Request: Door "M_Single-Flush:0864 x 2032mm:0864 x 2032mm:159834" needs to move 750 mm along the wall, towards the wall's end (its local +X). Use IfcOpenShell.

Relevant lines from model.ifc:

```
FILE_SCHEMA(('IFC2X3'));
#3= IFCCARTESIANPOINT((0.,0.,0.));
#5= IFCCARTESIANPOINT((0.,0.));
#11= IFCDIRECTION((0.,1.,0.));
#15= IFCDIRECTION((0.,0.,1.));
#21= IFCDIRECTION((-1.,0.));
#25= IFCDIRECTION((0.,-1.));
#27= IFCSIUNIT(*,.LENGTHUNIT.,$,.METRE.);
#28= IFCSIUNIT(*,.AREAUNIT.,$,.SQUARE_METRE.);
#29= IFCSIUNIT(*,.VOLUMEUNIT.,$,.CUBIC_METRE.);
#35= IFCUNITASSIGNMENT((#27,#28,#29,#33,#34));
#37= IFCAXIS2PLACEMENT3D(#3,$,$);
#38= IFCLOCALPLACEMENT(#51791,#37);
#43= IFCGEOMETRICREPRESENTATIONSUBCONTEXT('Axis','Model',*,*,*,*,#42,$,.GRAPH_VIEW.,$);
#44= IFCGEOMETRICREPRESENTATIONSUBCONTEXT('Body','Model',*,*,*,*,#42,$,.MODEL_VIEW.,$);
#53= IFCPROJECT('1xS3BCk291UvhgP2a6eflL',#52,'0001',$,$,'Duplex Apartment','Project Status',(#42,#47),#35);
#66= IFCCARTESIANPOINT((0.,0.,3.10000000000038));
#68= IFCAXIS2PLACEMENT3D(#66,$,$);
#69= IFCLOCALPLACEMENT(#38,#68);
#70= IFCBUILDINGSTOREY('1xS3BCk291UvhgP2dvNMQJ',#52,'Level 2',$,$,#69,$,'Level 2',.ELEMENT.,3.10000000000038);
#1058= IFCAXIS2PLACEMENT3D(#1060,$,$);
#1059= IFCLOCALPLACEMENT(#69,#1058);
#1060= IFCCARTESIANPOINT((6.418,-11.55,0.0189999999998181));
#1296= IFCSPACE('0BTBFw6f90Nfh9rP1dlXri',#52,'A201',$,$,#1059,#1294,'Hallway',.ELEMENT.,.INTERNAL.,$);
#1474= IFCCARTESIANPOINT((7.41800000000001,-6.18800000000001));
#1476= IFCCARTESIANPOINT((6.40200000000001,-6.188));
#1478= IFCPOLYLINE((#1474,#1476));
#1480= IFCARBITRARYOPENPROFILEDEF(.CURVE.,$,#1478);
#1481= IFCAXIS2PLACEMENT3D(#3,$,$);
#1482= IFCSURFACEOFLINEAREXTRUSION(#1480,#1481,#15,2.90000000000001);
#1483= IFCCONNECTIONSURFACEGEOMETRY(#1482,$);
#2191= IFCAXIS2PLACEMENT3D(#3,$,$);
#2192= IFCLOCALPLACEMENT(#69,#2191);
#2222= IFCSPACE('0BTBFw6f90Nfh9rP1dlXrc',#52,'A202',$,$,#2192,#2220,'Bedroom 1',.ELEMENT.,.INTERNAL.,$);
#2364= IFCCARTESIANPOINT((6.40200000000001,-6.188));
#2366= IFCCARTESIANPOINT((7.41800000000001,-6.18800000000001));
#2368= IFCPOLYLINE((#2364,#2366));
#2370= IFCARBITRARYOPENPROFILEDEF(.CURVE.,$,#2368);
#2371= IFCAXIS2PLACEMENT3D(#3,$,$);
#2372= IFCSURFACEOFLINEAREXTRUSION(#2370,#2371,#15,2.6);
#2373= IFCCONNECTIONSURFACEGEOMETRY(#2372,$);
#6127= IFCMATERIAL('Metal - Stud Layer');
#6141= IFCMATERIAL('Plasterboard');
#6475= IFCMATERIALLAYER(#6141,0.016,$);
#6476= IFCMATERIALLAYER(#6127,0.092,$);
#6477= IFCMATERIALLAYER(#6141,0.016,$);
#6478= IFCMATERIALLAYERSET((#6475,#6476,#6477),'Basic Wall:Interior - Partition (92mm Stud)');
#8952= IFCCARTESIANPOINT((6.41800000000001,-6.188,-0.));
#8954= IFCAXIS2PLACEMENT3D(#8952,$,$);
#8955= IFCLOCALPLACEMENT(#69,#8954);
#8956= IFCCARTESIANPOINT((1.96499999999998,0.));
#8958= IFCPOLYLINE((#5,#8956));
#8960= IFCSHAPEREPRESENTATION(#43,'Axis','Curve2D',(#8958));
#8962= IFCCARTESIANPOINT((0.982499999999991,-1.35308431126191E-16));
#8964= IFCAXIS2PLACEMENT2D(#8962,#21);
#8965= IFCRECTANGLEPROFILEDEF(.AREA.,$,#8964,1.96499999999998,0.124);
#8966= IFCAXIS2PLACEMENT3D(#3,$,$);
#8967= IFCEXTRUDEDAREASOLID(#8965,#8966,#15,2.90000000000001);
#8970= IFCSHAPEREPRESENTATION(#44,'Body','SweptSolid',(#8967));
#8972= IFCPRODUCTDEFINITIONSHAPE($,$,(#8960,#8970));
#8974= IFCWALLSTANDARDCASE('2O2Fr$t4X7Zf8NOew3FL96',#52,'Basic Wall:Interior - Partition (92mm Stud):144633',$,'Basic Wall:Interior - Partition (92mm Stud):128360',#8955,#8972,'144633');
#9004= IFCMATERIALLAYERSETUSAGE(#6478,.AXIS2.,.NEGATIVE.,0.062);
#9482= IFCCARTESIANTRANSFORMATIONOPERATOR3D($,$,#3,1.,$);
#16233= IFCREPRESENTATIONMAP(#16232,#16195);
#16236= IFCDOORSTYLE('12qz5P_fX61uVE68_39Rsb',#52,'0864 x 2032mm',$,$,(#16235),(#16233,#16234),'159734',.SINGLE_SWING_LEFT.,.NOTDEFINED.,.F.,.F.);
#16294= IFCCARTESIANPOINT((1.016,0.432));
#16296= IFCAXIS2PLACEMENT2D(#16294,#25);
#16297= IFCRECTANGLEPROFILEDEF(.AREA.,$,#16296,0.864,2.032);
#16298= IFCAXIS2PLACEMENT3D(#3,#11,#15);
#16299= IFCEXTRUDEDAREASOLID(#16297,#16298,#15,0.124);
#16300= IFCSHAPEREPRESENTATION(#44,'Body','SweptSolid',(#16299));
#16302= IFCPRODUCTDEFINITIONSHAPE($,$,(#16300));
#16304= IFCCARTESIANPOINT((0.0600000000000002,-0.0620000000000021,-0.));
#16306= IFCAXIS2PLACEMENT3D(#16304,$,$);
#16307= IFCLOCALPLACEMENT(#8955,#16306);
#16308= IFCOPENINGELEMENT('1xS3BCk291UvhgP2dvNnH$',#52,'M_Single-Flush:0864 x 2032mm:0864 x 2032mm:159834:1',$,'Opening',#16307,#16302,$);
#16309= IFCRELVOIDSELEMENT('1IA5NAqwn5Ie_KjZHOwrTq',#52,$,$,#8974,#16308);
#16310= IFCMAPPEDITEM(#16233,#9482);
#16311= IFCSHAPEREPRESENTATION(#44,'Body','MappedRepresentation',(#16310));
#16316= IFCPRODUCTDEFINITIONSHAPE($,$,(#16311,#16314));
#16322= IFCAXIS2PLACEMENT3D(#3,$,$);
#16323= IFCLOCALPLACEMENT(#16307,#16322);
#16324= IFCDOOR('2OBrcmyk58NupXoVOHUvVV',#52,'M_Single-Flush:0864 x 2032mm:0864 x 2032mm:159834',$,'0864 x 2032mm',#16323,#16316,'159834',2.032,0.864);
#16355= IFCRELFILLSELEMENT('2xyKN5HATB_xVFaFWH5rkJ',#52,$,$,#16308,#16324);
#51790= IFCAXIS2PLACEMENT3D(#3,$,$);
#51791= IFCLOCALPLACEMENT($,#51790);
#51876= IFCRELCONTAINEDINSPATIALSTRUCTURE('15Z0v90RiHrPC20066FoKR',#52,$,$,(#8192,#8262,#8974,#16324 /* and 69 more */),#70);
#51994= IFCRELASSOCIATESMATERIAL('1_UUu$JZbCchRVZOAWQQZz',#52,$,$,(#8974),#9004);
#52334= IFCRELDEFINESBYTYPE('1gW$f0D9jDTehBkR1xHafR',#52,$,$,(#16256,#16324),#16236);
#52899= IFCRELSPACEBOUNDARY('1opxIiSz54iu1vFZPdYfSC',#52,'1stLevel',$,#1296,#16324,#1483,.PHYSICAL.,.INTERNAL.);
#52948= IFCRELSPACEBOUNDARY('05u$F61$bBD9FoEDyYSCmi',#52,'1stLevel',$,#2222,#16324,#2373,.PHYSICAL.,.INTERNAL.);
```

```python
import numpy as np
import ifcopenshell
import ifcopenshell.api.geometry
import ifcopenshell.util.placement

model = ifcopenshell.open("model.ifc")

door = model.by_guid("2OBrcmyk58NupXoVOHUvVV")
opening = door.FillsVoids[0].RelatingOpeningElement
wall = opening.VoidsElements[0].RelatingBuildingElement

wall_matrix = ifcopenshell.util.placement.get_local_placement(wall.ObjectPlacement)
shift = wall_matrix[:3, 0] * 0.75
before = ifcopenshell.util.placement.get_local_placement(door.ObjectPlacement)[:3, 3].copy()

# The door is placed relative to its opening, so it follows when the opening moves.
matrix = ifcopenshell.util.placement.get_local_placement(opening.ObjectPlacement)
matrix[:3, 3] += shift
ifcopenshell.api.geometry.edit_object_placement(
    model, product=opening, matrix=matrix, is_si=False, should_transform_children=True
)

# Space boundary surfaces are stored in each space's coordinates; move them too.
for rel in door.ProvidesBoundaries:
    if not rel.ConnectionGeometry:
        continue
    surface = rel.ConnectionGeometry.SurfaceOnRelatingElement
    space_matrix = ifcopenshell.util.placement.get_local_placement(rel.RelatingSpace.ObjectPlacement)
    point = np.array(surface.Position.Location.Coordinates) + space_matrix[:3, :3].T @ shift
    surface.Position = model.createIfcAxis2Placement3D(
        model.createIfcCartesianPoint(point.tolist()), surface.Position.Axis, surface.Position.RefDirection
    )

after = ifcopenshell.util.placement.get_local_placement(door.ObjectPlacement)[:3, 3]
print("door moved by", (after - before).round(3) + 0.0)

model.write("model_edited.ifc")
```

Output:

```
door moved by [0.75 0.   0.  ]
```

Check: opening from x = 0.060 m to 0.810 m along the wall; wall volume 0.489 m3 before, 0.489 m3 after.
